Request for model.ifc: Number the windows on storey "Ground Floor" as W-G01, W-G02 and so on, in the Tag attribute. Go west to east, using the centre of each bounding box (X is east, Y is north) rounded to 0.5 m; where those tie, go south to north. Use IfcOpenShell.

First a look at what the model holds.

```python
import ifcopenshell
import ifcopenshell.util.element
import ifcopenshell.util.placement

model = ifcopenshell.open("model.ifc")
print(model.schema)
storey = next(s for s in model.by_type("IfcBuildingStorey") if s.Name == "Ground Floor")
windows = [e for e in ifcopenshell.util.element.get_decomposition(storey) if e.is_a("IfcWindow")]
for e in sorted(windows, key=lambda e: e.id()):
    origin = ifcopenshell.util.placement.get_local_placement(e.ObjectPlacement)[:3, 3]
    print(e.id(), e.Tag, e.Name, origin.round(2) + 0.0, sep=" | ")
```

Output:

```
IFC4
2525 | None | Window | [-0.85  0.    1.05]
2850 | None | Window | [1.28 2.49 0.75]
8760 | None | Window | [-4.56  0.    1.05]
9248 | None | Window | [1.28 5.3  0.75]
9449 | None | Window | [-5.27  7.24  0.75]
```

```python
import ifcopenshell
import ifcopenshell.geom
import ifcopenshell.util.element
import ifcopenshell.util.shape

model = ifcopenshell.open("model.ifc")
settings = ifcopenshell.geom.settings()
settings.set("use-world-coords", True)


def centre(element):
    shape = ifcopenshell.geom.create_shape(settings, element)
    return ifcopenshell.util.shape.get_bbox_centroid(shape.geometry)


storey = next(s for s in model.by_type("IfcBuildingStorey") if s.Name == "Ground Floor")
windows = [e for e in ifcopenshell.util.element.get_decomposition(storey) if e.is_a("IfcWindow")]

# Insertion points can sit at a corner or the storey origin, so sort by the geometry (in metres).
centres = {e: centre(e) for e in windows}
windows.sort(key=lambda e: (round(centres[e][0] / 0.5), centres[e][1]))

for i, e in enumerate(windows, start=1):
    number = f"W-G{i:02d}"
    e.Tag = number
    print(e.id(), number)

model.write("model-out.ifc")
```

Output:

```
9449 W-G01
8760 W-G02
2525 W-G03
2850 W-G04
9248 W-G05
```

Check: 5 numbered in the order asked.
